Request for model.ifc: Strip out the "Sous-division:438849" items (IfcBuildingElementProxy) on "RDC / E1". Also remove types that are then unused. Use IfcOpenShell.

First a look at what the model holds.

```python
import ifcopenshell
import ifcopenshell.util.element

model = ifcopenshell.open("model.ifc")
print(model.schema)
storey = next(s for s in model.by_type("IfcBuildingStorey") if s.Name == "RDC / E1")
proxies = [e for e in ifcopenshell.util.element.get_decomposition(storey) if e.is_a("IfcBuildingElementProxy")]
seen = {}
for e in proxies:
    element_type = ifcopenshell.util.element.get_type(e)
    name = element_type.Name if element_type not in (None, e) else None
    seen[name] = seen.get(name, 0) + 1
for name, count in sorted(seen.items(), key=str):
    print(count, "x", name)
```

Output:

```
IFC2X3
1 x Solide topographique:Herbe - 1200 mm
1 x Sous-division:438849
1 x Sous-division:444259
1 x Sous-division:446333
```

```python
import ifcopenshell
import ifcopenshell.api.root
import ifcopenshell.util.element

model = ifcopenshell.open("model.ifc")

storey = next(s for s in model.by_type("IfcBuildingStorey") if s.Name == "RDC / E1")
proxies = [e for e in ifcopenshell.util.element.get_decomposition(storey) if e.is_a("IfcBuildingElementProxy")]
targets = [e for e in proxies if (t := ifcopenshell.util.element.get_type(e)) not in (None, e) and t.Name == "Sous-division:438849"]
types = {ifcopenshell.util.element.get_type(e) for e in targets} - {None, *targets}

for e in targets:
    ifcopenshell.api.root.remove_product(model, product=e)
print(len(targets), "removed")

unused = [t for t in types if not ifcopenshell.util.element.get_types(t)]
for t in unused:
    ifcopenshell.api.root.remove_product(model, product=t)
print(len(unused), "unused types removed")

model.write("model_edited.ifc")
```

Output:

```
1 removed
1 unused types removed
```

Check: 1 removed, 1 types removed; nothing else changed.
